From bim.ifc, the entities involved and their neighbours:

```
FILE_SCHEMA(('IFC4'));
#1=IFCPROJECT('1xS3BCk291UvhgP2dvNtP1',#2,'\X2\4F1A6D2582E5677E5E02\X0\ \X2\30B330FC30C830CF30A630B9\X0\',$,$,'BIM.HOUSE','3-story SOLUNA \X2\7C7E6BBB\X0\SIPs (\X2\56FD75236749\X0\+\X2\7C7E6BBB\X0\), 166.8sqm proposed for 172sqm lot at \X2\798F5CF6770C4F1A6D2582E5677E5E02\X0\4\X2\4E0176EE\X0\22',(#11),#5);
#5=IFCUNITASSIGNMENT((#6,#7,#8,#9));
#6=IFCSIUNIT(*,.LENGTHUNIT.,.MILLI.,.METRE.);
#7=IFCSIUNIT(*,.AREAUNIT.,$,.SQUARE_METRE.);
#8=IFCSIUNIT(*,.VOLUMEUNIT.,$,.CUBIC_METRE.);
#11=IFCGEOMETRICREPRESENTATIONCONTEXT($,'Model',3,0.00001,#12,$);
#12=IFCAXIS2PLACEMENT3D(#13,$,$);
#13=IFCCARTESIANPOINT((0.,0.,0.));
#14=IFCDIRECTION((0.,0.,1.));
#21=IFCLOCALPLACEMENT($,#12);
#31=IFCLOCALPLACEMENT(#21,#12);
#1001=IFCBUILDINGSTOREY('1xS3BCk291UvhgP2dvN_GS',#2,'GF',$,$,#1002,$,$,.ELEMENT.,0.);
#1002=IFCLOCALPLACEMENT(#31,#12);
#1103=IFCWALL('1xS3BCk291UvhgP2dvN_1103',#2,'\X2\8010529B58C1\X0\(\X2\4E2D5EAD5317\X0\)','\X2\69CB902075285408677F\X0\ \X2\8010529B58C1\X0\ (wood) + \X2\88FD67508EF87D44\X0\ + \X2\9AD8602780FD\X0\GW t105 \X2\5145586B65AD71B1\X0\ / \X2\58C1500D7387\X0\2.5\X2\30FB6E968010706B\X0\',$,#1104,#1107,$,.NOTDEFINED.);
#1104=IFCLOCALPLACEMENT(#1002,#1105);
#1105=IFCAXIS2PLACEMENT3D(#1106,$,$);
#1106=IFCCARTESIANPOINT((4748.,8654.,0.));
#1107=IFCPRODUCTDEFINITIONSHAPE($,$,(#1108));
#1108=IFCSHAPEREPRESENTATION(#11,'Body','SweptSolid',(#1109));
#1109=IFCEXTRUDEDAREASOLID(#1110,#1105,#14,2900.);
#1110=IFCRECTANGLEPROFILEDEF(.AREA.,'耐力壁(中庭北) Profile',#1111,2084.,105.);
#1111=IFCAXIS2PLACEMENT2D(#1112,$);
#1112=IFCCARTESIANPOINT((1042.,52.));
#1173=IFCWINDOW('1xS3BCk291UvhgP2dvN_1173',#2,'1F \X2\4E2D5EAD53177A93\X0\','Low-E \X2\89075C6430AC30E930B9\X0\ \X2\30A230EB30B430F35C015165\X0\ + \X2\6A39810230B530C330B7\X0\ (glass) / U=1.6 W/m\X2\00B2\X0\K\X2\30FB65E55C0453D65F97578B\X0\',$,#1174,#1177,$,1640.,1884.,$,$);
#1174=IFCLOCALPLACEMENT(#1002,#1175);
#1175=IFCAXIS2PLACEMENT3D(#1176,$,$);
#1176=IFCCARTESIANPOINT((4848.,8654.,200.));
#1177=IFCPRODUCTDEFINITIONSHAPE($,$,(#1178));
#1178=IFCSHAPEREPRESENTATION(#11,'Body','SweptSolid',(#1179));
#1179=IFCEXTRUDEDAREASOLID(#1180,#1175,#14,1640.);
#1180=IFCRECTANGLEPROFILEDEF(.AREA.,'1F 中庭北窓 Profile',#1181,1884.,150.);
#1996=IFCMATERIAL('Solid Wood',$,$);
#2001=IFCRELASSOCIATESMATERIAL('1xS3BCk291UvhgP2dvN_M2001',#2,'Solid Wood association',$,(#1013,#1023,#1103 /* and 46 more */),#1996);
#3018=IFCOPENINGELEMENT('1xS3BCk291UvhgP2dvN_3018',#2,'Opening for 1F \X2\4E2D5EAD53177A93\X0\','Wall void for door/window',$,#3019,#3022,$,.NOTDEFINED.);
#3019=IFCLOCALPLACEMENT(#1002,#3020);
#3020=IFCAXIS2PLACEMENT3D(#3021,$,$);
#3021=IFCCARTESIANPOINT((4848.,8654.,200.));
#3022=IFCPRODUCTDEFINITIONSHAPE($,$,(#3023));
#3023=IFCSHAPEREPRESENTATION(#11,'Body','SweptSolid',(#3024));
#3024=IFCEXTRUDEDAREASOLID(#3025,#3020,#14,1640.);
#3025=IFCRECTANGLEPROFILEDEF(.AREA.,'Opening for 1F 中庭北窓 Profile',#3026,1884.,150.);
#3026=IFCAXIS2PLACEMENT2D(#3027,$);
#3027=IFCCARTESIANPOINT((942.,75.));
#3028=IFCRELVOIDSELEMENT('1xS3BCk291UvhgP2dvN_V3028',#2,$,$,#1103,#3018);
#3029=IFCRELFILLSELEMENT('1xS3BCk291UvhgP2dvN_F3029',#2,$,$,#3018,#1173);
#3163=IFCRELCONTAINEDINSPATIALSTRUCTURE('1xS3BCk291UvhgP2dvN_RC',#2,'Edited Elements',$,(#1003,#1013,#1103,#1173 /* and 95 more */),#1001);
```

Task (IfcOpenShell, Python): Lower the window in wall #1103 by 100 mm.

```python
import numpy as np
import ifcopenshell
import ifcopenshell.api.geometry
import ifcopenshell.util.placement
import ifcopenshell.util.unit

model = ifcopenshell.open("bim.ifc")
unit_scale = ifcopenshell.util.unit.calculate_unit_scale(model)

window = model.by_guid("1xS3BCk291UvhgP2dvN_1173")
opening = window.FillsVoids[0].RelatingOpeningElement
dz = -100.0

shift = np.array([0.0, 0.0, dz])
# The window is not placed relative to its opening, so move both.
for product in (opening, window):
    matrix = ifcopenshell.util.placement.get_local_placement(product.ObjectPlacement)
    matrix[:3, 3] += shift
    ifcopenshell.api.geometry.edit_object_placement(model, product=product, matrix=matrix, is_si=False)

print(f"moved by {dz * unit_scale:+.3f} m")

model.write("bim_v2.ifc")
```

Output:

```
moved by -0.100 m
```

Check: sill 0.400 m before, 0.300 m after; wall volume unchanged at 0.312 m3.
